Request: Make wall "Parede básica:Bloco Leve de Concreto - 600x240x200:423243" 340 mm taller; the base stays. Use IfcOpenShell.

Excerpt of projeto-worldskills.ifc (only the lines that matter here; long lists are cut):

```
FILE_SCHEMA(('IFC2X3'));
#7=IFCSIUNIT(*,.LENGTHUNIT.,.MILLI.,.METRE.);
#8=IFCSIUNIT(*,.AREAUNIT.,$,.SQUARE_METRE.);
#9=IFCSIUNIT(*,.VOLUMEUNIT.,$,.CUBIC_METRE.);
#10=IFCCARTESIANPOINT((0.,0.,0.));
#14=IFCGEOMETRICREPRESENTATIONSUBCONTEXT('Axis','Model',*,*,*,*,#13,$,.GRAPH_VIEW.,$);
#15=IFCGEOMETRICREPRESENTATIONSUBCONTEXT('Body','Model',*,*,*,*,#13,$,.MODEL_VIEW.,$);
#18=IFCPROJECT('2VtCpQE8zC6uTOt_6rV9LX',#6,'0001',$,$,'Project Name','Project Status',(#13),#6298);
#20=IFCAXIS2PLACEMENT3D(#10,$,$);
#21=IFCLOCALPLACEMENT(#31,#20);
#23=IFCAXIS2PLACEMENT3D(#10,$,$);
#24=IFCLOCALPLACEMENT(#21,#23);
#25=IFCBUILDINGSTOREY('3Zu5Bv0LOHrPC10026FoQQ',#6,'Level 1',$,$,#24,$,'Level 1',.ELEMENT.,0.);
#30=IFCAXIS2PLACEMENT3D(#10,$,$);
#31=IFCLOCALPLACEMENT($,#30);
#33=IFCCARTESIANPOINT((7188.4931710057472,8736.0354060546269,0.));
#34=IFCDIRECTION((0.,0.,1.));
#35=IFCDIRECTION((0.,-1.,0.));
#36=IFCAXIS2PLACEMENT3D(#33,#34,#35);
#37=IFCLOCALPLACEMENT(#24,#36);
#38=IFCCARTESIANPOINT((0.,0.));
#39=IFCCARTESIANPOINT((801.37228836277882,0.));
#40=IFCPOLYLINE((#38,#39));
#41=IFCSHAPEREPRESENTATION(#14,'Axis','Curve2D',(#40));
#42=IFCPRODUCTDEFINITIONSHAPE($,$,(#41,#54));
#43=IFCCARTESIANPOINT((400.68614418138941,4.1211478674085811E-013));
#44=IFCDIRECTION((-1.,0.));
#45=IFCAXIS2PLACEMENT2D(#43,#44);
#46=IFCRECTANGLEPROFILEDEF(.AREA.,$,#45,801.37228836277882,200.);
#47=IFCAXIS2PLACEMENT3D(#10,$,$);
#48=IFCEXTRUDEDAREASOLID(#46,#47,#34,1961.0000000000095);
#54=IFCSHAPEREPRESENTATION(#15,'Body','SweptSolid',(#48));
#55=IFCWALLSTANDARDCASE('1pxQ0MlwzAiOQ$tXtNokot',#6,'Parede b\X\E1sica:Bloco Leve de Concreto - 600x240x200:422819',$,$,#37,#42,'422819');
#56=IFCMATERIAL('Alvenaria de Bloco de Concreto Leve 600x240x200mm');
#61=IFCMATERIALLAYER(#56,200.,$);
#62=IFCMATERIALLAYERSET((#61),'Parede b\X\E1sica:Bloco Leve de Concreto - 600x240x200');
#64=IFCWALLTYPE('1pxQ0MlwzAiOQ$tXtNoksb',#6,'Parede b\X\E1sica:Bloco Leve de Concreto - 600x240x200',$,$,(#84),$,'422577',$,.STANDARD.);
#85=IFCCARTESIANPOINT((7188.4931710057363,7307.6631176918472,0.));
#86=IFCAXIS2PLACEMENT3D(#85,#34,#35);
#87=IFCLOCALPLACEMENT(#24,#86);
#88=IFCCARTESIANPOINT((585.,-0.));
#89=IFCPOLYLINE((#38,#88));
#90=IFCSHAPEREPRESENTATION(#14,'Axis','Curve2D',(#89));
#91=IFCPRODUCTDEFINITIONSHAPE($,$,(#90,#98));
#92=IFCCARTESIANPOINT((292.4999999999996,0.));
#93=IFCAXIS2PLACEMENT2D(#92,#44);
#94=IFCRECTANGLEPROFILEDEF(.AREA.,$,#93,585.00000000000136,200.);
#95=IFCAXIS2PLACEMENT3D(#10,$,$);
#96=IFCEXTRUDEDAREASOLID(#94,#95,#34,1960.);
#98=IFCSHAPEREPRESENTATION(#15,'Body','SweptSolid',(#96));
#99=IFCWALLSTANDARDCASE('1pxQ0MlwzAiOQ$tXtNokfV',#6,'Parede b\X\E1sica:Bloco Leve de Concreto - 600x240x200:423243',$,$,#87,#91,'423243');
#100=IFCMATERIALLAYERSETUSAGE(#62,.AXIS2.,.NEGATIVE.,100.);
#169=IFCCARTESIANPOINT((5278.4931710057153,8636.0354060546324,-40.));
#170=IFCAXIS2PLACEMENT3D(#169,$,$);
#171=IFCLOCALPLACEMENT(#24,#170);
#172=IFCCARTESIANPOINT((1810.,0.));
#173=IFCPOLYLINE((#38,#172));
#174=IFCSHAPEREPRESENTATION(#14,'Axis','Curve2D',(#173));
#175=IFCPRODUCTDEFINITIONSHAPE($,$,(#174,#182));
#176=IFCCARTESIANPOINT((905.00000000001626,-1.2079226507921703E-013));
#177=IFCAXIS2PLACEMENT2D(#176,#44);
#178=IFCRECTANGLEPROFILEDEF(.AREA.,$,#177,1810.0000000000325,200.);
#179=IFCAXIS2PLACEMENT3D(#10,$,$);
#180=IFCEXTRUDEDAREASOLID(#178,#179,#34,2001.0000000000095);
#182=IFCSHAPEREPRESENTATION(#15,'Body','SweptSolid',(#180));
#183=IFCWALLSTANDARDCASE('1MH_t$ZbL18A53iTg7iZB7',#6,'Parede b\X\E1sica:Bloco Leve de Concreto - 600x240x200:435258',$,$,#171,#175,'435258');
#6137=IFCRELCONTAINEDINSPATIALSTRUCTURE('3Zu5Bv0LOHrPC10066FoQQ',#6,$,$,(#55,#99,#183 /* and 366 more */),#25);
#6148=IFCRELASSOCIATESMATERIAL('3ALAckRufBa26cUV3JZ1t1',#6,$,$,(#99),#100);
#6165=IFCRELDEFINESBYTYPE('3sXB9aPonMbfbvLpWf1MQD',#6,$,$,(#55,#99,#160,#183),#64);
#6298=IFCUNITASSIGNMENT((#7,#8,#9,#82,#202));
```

```python
import ifcopenshell
import ifcopenshell.geom
import ifcopenshell.util.representation
import ifcopenshell.util.shape

model = ifcopenshell.open("projeto-worldskills.ifc")
settings = ifcopenshell.geom.settings()


def volume(element):
    """Net volume in cubic metres, openings subtracted."""
    shape = ifcopenshell.geom.create_shape(settings, element)
    return ifcopenshell.util.shape.get_volume(shape.geometry)


wall = model.by_guid("1pxQ0MlwzAiOQ$tXtNokfV")
before = volume(wall)

body = ifcopenshell.util.representation.get_representation(wall, "Model", "Body")
solid = body.Items[0]
old_height = solid.Depth
solid.Depth += 340.0
after = volume(wall)

print(f"height {old_height:g} -> {solid.Depth:g}, volume {before:.3f} -> {after:.3f} m3")

model.write("projeto-worldskills-out.ifc")
```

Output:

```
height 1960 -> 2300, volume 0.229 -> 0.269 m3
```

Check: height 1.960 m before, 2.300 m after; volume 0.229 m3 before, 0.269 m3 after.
